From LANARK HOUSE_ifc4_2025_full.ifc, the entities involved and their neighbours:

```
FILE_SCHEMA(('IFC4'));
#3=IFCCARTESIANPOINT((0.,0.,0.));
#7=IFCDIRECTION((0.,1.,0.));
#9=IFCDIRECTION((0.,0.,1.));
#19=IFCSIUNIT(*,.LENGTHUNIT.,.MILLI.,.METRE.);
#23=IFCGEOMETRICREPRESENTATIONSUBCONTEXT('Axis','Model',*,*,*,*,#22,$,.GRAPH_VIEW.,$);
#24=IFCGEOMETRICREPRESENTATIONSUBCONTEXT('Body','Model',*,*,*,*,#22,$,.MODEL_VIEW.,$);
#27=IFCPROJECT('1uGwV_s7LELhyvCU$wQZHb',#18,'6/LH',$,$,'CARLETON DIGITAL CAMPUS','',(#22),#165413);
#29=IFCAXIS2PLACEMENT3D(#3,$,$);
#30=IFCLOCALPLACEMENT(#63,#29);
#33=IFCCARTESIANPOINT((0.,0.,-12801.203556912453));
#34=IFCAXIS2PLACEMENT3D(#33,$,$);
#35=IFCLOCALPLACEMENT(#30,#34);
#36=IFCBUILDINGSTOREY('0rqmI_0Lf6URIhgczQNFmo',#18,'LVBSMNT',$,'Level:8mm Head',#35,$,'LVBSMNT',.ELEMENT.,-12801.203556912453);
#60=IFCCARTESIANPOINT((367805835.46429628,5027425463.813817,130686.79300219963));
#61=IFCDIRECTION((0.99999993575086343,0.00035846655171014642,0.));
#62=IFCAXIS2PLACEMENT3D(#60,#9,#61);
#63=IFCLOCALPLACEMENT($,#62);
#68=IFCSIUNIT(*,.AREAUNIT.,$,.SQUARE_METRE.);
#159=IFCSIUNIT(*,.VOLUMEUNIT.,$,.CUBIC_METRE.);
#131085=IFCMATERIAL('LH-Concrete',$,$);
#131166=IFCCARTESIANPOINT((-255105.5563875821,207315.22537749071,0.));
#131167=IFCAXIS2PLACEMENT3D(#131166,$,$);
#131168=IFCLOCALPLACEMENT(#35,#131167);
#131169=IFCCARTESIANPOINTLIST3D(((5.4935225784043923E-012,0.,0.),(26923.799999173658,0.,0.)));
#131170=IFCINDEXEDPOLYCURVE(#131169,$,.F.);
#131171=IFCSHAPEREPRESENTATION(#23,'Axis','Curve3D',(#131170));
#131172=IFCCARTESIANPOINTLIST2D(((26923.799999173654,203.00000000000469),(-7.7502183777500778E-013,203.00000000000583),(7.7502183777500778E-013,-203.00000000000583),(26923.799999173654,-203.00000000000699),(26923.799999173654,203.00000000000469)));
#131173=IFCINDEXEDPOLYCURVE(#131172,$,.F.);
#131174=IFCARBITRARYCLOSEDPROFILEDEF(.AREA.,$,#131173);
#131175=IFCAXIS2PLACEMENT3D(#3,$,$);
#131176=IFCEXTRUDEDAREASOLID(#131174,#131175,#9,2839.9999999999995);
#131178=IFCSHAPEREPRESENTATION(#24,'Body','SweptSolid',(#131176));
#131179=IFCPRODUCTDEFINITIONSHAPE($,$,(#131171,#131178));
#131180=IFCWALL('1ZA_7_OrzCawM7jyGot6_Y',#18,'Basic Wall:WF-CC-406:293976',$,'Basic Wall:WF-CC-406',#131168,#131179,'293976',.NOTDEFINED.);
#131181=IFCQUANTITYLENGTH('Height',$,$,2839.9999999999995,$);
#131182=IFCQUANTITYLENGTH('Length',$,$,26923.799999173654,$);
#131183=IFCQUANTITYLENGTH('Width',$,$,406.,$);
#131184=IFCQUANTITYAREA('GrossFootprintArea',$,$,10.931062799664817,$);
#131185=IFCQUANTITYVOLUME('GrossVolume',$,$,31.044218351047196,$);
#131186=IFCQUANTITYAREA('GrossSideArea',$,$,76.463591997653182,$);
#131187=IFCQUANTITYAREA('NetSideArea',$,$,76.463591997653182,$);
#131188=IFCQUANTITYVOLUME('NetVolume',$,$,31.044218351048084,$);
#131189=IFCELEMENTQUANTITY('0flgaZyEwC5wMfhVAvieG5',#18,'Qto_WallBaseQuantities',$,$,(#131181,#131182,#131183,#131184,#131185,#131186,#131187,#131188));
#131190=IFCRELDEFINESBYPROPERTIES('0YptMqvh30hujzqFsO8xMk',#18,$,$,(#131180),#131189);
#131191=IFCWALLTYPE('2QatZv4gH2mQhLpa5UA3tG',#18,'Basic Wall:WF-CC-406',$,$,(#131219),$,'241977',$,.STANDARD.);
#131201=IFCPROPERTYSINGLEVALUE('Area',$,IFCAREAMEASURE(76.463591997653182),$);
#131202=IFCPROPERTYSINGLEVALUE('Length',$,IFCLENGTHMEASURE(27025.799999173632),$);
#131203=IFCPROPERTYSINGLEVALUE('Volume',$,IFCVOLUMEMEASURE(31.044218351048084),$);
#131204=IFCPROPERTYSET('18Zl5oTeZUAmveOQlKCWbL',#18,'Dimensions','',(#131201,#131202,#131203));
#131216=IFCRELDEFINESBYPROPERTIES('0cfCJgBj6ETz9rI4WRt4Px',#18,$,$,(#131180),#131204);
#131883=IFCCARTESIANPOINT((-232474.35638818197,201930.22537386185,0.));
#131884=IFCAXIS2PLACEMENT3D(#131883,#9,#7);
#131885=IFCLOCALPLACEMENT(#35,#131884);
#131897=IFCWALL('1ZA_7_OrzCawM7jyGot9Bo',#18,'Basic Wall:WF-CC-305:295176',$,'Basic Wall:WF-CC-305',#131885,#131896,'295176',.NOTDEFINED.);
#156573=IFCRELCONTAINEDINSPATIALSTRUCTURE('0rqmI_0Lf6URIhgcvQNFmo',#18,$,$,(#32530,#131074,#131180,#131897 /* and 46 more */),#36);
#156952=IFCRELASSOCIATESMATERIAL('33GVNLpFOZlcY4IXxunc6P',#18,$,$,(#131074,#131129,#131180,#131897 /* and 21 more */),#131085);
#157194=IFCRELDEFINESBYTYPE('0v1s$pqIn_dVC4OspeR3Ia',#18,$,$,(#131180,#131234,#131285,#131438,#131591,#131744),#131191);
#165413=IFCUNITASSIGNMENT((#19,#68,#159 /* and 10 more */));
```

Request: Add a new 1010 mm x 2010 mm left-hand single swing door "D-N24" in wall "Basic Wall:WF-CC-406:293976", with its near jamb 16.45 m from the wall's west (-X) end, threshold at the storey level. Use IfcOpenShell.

```python
import numpy as np
import ifcopenshell
import ifcopenshell.api.feature
import ifcopenshell.api.geometry
import ifcopenshell.api.pset
import ifcopenshell.api.root
import ifcopenshell.api.spatial
import ifcopenshell.geom
import ifcopenshell.util.element
import ifcopenshell.util.placement
import ifcopenshell.util.representation
import ifcopenshell.util.shape
import ifcopenshell.util.unit

model = ifcopenshell.open("LANARK HOUSE_ifc4_2025_full.ifc")
unit_scale = ifcopenshell.util.unit.calculate_unit_scale(model)
area_scale = ifcopenshell.util.unit.calculate_unit_scale(model, "AREAUNIT")
volume_scale = ifcopenshell.util.unit.calculate_unit_scale(model, "VOLUMEUNIT")
settings = ifcopenshell.geom.settings()


def volume(element):
    """Net volume in cubic metres, openings subtracted."""
    shape = ifcopenshell.geom.create_shape(settings, element)
    return ifcopenshell.util.shape.get_volume(shape.geometry)


wall = model.by_guid("1ZA_7_OrzCawM7jyGot6_Y")
storey = ifcopenshell.util.element.get_container(wall, ifc_class="IfcBuildingStorey")
context = ifcopenshell.util.representation.get_context(model, "Model", "Body", "MODEL_VIEW")
before = volume(wall)

width, height, from_end, sill = 1.01, 2.01, 16.45, 0.0  # metres

# The wall runs along its own X axis, and the end named is its -X end.
wall_shape = ifcopenshell.geom.create_shape(settings, wall)
x, y, z = ifcopenshell.util.shape.get_vertices(wall_shape.geometry).T
start = x.min() + from_end
face, thickness = float(y.min()), float(y.max() - y.min())
wall_matrix = ifcopenshell.util.placement.get_local_placement(wall.ObjectPlacement)
level = ifcopenshell.util.placement.get_local_placement(storey.ObjectPlacement)[2, 3]


def in_wall(x, y):
    """Placement at x, y metres in the wall's axes, at sill height."""
    matrix = wall_matrix.copy()
    matrix[:, 3] = wall_matrix @ np.array([x / unit_scale, y / unit_scale, 0.0, 1.0])
    matrix[2, 3] = level + sill / unit_scale
    return matrix


# Opening: a box that overshoots both wall faces by 50 mm.
opening = ifcopenshell.api.root.create_entity(model, ifc_class="IfcOpeningElement", predefined_type="OPENING")
box = ifcopenshell.api.geometry.add_wall_representation(
    model, context=context, length=width, height=height, thickness=thickness + 0.1
)
ifcopenshell.api.geometry.assign_representation(model, product=opening, representation=box)
ifcopenshell.api.geometry.edit_object_placement(model, product=opening, matrix=in_wall(start, face - 0.05), is_si=False)
ifcopenshell.api.feature.add_feature(model, feature=opening, element=wall)

door = ifcopenshell.api.root.create_entity(model, ifc_class="IfcDoor", name="D-N24", predefined_type="DOOR")
door.OverallWidth, door.OverallHeight = width / unit_scale, height / unit_scale
door.OperationType = "SINGLE_SWING_LEFT"
body = ifcopenshell.api.geometry.add_door_representation(
    model,
    context=context,
    overall_width=door.OverallWidth,
    overall_height=door.OverallHeight,
    operation_type="SINGLE_SWING_LEFT",
    lining_properties={"LiningDepth": thickness / unit_scale, "ThresholdDepth": thickness / unit_scale},
)
ifcopenshell.api.geometry.assign_representation(model, product=door, representation=body)
ifcopenshell.api.spatial.assign_container(model, products=[door], relating_structure=storey)
ifcopenshell.api.feature.add_filling(model, opening=opening, element=door)

# The lining spans the wall, so the door starts at the wall face.
ifcopenshell.api.geometry.edit_object_placement(model, product=door, matrix=in_wall(start, face), is_si=False)

after = volume(wall)

# Update the wall's stored quantities.
qto = model.by_id(ifcopenshell.util.element.get_pset(wall, "Qto_WallBaseQuantities", should_inherit=False)["id"])
ifcopenshell.api.pset.edit_qto(model, qto=qto, properties={
    "NetSideArea": after / thickness / area_scale,
    "NetVolume": after / volume_scale,
})
pset = model.by_id(ifcopenshell.util.element.get_pset(wall, "Dimensions", should_inherit=False)["id"])
ifcopenshell.api.pset.edit_pset(model, pset=pset, properties={
    "Area": model.create_entity("IfcAreaMeasure", after / thickness / area_scale),
    "Volume": model.create_entity("IfcVolumeMeasure", after / volume_scale),
})

print(f"wall volume {before:.3f} -> {after:.3f} m3")

model.write("LANARK HOUSE_ifc4_2025_full_v2.ifc")
```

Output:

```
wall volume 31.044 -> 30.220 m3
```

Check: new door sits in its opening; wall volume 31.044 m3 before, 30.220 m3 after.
